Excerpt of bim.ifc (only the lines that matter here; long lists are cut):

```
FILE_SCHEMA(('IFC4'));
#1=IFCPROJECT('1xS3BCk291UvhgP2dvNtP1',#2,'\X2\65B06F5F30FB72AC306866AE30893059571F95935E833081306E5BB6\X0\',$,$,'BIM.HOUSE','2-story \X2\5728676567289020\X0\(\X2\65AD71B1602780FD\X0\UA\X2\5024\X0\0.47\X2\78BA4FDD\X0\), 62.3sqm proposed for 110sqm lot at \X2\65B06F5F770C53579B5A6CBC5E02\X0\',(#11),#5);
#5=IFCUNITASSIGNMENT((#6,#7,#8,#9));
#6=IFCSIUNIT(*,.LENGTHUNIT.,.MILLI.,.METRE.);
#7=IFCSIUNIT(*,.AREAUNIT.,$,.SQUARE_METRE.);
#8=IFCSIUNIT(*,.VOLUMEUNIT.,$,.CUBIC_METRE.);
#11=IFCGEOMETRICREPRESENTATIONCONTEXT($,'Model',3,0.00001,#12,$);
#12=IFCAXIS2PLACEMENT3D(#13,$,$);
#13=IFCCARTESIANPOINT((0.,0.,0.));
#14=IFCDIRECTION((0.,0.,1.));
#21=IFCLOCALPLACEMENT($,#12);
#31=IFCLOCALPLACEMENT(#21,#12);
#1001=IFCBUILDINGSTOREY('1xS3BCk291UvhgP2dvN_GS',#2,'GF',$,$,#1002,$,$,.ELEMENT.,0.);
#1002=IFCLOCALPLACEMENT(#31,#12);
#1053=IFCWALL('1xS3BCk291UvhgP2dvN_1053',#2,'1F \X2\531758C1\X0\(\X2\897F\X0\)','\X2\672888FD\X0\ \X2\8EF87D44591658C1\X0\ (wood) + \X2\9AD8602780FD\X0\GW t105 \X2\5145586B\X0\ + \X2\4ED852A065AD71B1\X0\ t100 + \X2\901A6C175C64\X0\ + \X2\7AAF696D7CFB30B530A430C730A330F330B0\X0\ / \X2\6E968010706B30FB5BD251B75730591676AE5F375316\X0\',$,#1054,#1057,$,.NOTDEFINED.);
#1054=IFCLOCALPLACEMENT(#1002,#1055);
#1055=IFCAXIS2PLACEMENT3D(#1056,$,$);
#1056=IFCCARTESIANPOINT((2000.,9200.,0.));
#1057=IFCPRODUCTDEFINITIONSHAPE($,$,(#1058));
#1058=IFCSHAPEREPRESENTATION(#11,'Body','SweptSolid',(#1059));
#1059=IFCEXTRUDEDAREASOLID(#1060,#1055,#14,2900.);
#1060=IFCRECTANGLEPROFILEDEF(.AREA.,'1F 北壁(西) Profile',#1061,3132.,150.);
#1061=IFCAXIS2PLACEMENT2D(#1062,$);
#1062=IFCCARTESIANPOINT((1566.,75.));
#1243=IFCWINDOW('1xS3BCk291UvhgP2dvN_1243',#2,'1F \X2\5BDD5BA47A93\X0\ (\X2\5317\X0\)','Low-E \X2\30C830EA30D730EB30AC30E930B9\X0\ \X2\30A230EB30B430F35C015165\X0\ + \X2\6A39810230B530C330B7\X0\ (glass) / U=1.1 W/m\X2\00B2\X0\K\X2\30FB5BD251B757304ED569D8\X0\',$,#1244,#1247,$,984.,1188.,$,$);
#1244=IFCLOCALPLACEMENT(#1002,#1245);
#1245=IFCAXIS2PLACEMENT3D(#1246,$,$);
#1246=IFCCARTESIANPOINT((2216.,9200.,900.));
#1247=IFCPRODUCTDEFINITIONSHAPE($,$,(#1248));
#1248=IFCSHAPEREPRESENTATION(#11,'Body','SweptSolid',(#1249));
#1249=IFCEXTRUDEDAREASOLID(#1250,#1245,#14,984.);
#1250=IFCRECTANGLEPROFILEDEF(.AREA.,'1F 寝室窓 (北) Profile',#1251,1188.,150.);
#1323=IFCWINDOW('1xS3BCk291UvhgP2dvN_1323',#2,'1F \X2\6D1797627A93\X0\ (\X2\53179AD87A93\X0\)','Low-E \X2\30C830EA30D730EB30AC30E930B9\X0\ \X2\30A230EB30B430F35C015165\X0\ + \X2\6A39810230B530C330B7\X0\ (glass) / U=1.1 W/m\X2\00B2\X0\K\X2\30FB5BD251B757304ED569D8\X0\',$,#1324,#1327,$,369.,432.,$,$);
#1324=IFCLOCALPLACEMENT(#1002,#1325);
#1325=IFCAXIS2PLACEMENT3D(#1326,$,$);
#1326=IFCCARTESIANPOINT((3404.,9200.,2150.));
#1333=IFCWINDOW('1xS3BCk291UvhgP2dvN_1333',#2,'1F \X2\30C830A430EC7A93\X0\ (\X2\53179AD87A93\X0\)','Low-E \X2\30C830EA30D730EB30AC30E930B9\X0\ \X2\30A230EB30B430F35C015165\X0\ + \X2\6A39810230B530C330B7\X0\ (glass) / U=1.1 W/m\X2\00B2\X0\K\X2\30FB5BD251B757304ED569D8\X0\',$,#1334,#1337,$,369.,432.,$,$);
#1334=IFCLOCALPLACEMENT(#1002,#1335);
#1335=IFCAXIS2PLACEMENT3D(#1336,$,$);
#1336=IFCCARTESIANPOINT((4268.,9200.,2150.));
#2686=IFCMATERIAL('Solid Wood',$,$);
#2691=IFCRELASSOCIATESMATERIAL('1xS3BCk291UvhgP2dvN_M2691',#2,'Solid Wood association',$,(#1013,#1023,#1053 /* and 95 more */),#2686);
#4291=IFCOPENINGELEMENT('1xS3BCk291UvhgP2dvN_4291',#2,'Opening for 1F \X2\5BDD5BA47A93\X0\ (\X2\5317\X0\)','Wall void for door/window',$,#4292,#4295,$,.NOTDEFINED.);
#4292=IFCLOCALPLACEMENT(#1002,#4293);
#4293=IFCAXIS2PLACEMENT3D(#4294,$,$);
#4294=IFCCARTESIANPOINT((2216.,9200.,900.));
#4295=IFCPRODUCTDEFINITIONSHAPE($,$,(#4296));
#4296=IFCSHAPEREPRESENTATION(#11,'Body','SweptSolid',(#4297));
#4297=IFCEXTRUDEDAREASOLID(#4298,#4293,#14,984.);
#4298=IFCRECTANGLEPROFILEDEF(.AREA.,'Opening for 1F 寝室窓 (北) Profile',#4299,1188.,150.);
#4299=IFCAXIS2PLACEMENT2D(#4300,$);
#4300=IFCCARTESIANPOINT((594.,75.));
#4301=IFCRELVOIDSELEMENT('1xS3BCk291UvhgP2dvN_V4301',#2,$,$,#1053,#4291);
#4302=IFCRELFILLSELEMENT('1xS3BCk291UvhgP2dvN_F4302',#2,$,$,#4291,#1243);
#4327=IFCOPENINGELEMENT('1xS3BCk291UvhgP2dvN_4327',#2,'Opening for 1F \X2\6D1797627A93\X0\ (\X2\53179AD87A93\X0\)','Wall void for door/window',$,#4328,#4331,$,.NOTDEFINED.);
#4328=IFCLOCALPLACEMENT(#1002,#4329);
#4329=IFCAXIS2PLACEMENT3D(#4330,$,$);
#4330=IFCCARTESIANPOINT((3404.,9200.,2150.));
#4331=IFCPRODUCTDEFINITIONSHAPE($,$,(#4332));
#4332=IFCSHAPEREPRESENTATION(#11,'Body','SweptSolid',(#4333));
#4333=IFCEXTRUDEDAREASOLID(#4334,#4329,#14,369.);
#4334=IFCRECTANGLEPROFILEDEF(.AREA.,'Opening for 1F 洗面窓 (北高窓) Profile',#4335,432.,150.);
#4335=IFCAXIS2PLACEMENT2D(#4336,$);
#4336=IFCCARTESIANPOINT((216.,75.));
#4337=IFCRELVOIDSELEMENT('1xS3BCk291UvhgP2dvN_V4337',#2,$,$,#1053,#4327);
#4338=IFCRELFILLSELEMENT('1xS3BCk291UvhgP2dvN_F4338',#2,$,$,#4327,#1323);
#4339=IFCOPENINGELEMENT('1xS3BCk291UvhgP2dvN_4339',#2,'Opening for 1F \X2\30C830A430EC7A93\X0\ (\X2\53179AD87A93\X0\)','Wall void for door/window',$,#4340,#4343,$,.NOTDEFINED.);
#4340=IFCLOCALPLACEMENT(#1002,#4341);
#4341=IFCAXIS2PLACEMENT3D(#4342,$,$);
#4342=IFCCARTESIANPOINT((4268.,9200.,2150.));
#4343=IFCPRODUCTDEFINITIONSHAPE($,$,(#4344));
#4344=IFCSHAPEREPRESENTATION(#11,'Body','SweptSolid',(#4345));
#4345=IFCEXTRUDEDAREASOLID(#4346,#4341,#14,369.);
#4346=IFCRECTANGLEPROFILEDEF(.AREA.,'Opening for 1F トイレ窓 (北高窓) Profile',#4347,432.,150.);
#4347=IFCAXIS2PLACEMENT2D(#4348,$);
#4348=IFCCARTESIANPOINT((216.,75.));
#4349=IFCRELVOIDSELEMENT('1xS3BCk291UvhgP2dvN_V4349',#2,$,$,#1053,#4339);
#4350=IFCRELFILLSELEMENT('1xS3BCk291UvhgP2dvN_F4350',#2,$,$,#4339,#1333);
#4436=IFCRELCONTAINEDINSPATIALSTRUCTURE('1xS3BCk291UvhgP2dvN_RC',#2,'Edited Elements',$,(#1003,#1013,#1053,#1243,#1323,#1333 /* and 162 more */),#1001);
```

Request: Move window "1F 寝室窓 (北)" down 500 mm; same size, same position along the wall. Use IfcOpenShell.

```python
import numpy as np
import ifcopenshell
import ifcopenshell.api.geometry
import ifcopenshell.util.placement
import ifcopenshell.util.unit

model = ifcopenshell.open("bim.ifc")
unit_scale = ifcopenshell.util.unit.calculate_unit_scale(model)

window = model.by_id(1243)
opening = window.FillsVoids[0].RelatingOpeningElement
dz = -0.5 / unit_scale

shift = np.array([0.0, 0.0, dz])
# The window is not placed relative to its opening, so move both.
for product in (opening, window):
    matrix = ifcopenshell.util.placement.get_local_placement(product.ObjectPlacement)
    matrix[:3, 3] += shift
    ifcopenshell.api.geometry.edit_object_placement(model, product=product, matrix=matrix, is_si=False)

print(f"moved by {dz * unit_scale:+.3f} m")

model.write("bim_rev.ifc")
```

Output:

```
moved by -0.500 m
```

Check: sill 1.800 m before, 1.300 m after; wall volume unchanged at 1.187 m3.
